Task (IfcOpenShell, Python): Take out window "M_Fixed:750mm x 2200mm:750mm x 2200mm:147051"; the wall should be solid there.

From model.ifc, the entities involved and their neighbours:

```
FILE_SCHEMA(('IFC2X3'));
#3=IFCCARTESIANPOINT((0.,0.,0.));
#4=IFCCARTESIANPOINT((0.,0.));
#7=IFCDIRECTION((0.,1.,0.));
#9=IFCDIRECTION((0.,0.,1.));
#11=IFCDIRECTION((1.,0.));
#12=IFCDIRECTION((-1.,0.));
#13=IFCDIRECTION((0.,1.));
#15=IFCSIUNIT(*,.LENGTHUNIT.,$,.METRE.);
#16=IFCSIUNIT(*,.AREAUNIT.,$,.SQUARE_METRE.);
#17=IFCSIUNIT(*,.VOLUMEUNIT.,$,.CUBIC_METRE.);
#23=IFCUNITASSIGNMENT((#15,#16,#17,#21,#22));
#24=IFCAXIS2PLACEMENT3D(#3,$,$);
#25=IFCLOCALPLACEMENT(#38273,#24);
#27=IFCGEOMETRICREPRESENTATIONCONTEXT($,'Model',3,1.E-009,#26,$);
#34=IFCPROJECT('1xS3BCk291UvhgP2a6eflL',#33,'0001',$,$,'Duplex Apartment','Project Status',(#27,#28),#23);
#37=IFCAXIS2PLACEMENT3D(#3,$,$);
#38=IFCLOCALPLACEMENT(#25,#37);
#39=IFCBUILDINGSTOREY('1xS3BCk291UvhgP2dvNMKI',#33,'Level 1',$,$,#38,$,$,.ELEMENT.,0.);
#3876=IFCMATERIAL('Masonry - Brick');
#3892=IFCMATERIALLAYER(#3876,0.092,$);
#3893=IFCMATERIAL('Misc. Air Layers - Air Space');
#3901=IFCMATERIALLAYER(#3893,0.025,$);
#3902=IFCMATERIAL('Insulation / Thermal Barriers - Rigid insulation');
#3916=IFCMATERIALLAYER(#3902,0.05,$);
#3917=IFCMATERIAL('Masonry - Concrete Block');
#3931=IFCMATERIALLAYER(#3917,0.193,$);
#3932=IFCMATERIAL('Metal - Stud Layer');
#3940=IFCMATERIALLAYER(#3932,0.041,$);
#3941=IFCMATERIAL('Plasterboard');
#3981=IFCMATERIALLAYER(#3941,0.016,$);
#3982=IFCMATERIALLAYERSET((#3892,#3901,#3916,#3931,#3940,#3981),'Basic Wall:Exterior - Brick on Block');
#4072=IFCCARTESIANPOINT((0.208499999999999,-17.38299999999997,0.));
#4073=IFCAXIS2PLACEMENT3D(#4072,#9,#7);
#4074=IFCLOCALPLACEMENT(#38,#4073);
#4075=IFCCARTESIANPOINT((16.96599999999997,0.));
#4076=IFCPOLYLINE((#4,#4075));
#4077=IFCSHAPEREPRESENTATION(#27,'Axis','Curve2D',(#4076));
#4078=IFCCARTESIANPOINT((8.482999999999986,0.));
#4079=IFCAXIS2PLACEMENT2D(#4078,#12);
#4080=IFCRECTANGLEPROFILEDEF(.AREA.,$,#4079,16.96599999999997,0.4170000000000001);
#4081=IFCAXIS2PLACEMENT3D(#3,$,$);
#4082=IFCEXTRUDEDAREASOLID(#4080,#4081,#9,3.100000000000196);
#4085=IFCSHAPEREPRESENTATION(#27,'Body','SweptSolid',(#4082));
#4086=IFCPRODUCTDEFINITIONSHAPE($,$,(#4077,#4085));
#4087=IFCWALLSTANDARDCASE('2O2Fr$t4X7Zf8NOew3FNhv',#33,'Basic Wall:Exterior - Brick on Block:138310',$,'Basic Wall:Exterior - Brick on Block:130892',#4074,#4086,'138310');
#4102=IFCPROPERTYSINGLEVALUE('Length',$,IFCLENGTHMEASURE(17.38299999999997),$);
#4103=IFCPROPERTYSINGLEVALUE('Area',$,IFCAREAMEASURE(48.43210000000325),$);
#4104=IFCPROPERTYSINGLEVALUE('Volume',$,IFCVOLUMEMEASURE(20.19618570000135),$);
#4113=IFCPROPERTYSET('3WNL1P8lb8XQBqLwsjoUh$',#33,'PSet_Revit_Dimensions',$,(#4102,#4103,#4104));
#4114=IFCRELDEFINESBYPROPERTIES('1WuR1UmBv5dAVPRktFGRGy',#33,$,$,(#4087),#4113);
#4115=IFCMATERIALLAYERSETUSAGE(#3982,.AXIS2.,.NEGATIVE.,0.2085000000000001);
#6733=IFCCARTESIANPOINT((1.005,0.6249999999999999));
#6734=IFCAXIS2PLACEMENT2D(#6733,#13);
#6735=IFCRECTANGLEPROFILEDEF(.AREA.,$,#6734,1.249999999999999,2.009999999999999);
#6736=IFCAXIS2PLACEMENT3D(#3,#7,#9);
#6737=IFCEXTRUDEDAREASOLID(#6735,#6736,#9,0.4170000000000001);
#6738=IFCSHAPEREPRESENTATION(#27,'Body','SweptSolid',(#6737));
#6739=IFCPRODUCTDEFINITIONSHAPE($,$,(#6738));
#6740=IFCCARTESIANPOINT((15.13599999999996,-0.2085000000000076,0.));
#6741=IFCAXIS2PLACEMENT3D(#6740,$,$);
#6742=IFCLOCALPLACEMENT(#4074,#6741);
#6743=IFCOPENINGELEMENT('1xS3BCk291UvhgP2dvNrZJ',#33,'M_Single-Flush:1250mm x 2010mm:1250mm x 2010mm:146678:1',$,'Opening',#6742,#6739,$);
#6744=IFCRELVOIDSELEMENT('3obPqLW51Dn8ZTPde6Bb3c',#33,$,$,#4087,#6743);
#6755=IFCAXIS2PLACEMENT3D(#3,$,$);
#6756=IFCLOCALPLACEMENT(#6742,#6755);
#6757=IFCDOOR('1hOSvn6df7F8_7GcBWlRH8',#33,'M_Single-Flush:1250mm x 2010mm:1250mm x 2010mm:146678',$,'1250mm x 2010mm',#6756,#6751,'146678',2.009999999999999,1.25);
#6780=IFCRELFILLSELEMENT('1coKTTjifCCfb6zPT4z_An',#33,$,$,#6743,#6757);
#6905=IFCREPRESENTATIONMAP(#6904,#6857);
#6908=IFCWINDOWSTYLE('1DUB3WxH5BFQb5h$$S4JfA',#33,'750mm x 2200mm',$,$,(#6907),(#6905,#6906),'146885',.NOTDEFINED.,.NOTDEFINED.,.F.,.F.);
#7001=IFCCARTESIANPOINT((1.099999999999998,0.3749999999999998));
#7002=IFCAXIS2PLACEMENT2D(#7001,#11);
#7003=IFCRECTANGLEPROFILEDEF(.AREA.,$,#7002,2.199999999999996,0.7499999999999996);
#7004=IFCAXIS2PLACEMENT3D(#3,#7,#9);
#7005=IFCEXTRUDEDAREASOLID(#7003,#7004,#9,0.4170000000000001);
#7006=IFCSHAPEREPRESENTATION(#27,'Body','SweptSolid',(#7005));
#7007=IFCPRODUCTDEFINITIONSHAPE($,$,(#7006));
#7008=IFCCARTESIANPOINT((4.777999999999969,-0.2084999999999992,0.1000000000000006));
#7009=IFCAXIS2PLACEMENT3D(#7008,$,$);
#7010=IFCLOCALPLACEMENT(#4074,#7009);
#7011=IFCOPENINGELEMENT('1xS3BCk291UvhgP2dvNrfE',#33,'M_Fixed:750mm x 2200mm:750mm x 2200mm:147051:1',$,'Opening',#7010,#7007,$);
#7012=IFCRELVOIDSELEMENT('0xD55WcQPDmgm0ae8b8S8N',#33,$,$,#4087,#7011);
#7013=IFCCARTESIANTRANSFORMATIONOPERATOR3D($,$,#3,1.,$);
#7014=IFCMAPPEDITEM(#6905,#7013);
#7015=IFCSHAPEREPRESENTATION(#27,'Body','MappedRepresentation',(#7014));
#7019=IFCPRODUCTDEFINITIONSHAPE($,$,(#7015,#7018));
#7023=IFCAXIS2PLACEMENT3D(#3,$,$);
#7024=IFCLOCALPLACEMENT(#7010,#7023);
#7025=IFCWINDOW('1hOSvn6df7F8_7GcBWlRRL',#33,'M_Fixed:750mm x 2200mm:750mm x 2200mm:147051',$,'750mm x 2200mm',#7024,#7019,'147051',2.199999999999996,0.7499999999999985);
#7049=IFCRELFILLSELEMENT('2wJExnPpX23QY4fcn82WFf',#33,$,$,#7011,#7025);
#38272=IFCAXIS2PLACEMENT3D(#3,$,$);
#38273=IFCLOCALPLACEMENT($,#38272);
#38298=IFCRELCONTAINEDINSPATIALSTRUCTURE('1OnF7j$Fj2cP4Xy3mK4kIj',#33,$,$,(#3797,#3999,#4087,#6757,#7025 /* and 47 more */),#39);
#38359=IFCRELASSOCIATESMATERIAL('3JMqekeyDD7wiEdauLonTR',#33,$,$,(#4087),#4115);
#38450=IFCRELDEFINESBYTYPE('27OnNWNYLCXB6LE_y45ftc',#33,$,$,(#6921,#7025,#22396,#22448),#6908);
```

```python
import ifcopenshell
import ifcopenshell.api.feature
import ifcopenshell.api.pset
import ifcopenshell.api.root
import ifcopenshell.geom
import ifcopenshell.util.element
import ifcopenshell.util.shape
import ifcopenshell.util.unit

model = ifcopenshell.open("model.ifc")
area_scale = ifcopenshell.util.unit.calculate_unit_scale(model, "AREAUNIT")
volume_scale = ifcopenshell.util.unit.calculate_unit_scale(model, "VOLUMEUNIT")
settings = ifcopenshell.geom.settings()


def volume(element):
    """Net volume in cubic metres, openings subtracted."""
    shape = ifcopenshell.geom.create_shape(settings, element)
    return ifcopenshell.util.shape.get_volume(shape.geometry)


window = model.by_guid("1hOSvn6df7F8_7GcBWlRRL")
opening = window.FillsVoids[0].RelatingOpeningElement
wall = opening.VoidsElements[0].RelatingBuildingElement
before = volume(wall)

ifcopenshell.api.root.remove_product(model, product=window)
ifcopenshell.api.feature.remove_feature(model, feature=opening)

after = volume(wall)
thickness = 0.417  # wall thickness in metres

# Update the wall's stored quantities.
pset = model.by_id(ifcopenshell.util.element.get_pset(wall, "PSet_Revit_Dimensions", should_inherit=False)["id"])
ifcopenshell.api.pset.edit_pset(model, pset=pset, properties={
    "Area": model.create_entity("IfcAreaMeasure", after / thickness / area_scale),
    "Volume": model.create_entity("IfcVolumeMeasure", after / volume_scale),
})

print(f"wall volume {before:.3f} -> {after:.3f} m3")

model.write("model_edited.ifc")
```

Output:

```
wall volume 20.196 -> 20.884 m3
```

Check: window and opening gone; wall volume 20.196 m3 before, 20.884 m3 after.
